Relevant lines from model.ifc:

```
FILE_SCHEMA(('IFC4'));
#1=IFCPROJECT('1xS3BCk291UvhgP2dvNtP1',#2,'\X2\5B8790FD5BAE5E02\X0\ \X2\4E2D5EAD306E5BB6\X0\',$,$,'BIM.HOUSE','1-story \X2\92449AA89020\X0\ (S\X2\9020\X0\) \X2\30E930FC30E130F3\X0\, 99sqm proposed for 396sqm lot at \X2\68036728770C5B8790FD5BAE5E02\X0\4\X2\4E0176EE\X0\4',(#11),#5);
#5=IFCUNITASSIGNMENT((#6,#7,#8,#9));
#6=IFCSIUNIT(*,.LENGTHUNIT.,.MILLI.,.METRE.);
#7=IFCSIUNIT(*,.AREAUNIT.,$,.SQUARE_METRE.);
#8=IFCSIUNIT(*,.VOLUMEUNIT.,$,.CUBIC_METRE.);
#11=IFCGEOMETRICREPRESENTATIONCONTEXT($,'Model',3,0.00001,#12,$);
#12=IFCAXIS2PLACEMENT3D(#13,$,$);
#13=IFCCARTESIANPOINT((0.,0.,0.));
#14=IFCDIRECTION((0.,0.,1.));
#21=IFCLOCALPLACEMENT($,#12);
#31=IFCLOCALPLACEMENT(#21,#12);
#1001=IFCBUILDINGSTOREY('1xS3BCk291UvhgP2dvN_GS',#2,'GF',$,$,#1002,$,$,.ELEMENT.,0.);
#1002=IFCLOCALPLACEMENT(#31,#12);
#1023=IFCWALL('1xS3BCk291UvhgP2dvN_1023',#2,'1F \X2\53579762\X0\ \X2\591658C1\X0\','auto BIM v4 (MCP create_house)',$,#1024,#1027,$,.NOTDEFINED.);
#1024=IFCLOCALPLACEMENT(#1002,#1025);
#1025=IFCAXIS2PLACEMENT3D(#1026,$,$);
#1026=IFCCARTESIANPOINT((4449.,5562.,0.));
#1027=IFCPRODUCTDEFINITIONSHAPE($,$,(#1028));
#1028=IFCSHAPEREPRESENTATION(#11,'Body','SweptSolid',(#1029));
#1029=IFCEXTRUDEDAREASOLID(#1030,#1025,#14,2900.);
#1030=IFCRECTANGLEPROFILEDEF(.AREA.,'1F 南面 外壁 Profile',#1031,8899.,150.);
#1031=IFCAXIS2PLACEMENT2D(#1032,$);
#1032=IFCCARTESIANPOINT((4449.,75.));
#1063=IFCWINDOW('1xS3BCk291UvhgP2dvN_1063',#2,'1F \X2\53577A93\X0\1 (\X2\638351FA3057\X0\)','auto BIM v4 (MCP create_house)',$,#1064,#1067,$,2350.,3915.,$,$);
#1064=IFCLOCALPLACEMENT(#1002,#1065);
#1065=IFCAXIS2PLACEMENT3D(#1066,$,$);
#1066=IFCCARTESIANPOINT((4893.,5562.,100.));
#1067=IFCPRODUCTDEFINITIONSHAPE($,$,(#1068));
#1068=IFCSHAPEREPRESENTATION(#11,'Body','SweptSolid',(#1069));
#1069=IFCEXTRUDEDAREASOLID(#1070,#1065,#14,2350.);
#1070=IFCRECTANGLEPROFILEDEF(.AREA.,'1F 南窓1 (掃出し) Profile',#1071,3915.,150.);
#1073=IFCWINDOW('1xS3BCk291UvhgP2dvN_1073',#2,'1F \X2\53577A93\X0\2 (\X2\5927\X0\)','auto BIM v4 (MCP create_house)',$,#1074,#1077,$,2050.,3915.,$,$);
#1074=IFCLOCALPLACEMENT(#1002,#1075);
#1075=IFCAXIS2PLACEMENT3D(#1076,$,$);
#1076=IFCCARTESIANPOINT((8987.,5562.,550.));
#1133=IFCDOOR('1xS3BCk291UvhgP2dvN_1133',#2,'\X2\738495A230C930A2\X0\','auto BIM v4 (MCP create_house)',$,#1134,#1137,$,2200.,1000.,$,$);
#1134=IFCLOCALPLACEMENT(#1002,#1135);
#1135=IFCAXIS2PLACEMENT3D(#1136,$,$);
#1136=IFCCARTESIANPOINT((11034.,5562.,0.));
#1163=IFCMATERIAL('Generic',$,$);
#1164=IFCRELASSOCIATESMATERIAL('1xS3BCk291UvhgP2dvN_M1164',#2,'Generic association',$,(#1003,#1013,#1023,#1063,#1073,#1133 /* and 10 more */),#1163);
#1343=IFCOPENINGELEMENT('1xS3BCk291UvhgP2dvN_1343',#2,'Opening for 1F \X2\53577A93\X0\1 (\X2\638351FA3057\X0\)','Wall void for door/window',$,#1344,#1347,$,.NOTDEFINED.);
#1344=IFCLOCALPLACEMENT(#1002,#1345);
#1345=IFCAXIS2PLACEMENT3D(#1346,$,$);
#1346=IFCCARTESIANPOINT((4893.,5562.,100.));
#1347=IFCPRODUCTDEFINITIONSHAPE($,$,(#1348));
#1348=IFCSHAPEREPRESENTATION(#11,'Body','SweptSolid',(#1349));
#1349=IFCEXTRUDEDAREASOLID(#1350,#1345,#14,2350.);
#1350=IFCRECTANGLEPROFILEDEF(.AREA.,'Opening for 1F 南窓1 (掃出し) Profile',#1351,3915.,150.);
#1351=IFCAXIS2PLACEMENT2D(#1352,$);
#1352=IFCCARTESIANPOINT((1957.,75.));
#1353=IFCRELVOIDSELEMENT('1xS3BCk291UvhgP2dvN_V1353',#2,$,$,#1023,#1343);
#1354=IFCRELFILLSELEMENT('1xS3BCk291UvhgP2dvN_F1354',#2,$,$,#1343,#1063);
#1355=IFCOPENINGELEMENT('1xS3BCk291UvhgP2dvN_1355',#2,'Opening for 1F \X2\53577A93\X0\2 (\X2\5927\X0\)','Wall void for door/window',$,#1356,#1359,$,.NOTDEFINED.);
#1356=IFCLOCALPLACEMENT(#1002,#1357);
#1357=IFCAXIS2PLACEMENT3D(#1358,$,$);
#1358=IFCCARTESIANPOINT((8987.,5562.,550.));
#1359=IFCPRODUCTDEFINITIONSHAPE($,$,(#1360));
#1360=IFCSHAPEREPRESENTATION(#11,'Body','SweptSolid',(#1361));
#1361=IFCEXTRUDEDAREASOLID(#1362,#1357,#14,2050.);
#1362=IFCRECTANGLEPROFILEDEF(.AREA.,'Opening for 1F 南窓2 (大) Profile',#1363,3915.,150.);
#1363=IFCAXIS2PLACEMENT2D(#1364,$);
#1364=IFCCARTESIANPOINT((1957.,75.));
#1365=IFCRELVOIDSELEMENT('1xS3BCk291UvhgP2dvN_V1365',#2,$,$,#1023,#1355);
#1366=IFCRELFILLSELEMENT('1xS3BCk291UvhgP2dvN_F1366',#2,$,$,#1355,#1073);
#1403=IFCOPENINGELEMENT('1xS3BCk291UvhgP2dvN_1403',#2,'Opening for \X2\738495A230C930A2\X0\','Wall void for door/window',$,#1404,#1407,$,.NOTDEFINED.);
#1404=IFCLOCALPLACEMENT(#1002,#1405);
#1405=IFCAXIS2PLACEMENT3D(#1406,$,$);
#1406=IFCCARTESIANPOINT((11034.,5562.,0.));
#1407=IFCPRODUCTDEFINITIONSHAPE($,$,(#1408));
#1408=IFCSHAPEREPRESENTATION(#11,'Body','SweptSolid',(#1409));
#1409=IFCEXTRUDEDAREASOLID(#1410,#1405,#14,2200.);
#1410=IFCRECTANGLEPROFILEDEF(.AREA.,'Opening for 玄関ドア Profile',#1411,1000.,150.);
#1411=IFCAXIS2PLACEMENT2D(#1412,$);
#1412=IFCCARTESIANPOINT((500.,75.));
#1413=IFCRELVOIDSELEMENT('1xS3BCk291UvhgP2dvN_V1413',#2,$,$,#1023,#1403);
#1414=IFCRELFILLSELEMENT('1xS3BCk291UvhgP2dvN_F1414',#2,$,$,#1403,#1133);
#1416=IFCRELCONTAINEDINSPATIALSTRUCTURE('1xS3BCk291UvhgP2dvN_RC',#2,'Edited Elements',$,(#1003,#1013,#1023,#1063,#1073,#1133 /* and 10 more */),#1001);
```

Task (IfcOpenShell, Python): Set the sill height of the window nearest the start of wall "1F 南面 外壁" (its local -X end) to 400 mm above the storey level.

```python
import numpy as np
import ifcopenshell
import ifcopenshell.api.geometry
import ifcopenshell.geom
import ifcopenshell.util.element
import ifcopenshell.util.placement
import ifcopenshell.util.shape
import ifcopenshell.util.unit

model = ifcopenshell.open("model.ifc")
unit_scale = ifcopenshell.util.unit.calculate_unit_scale(model)

window = model.by_guid("1xS3BCk291UvhgP2dvN_1063")
opening = window.FillsVoids[0].RelatingOpeningElement
storey = ifcopenshell.util.element.get_container(window, ifc_class="IfcBuildingStorey")
level = ifcopenshell.util.placement.get_local_placement(storey.ObjectPlacement)[2, 3]

# The opening's origin need not be at the sill, so measure its lowest point.
shape = ifcopenshell.geom.create_shape(ifcopenshell.geom.settings(), opening)
bottom = ifcopenshell.util.shape.get_shape_bottom_elevation(shape, shape.geometry) / unit_scale
dz = level + 400.0 - bottom

shift = np.array([0.0, 0.0, dz])
# The window is not placed relative to its opening, so move both.
for product in (opening, window):
    matrix = ifcopenshell.util.placement.get_local_placement(product.ObjectPlacement)
    matrix[:3, 3] += shift
    ifcopenshell.api.geometry.edit_object_placement(model, product=product, matrix=matrix, is_si=False)

print(f"moved by {dz * unit_scale:+.3f} m")

model.write("model-out.ifc")
```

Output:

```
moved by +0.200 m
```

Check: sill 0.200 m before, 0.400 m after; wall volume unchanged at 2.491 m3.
